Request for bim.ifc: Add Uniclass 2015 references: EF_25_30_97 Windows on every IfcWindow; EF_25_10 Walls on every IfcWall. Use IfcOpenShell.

First a look at what the model holds.

```python
import ifcopenshell

model = ifcopenshell.open("bim.ifc")
print(model.schema)
print("classifications:", [c.Name for c in model.by_type("IfcClassification")])
for ifc_class in ("IfcDoor", "IfcRoof", "IfcStair", "IfcWall", "IfcWindow"):
    print(ifc_class, len(model.by_type(ifc_class)))
```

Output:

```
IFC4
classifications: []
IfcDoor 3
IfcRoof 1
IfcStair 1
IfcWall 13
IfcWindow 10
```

```python
import ifcopenshell
import ifcopenshell.api.classification

model = ifcopenshell.open("bim.ifc")

system = ifcopenshell.api.classification.add_classification(model, classification="Uniclass 2015")

codes = {
    "IfcWindow": ("EF_25_30_97", "Windows"),
    "IfcWall": ("EF_25_10", "Walls"),
}
for ifc_class, (code, name) in codes.items():
    products = model.by_type(ifc_class)
    ifcopenshell.api.classification.add_reference(
        model, products=products, classification=system, identification=code, name=name
    )
    print(code, len(products))

model.write("bim_v2.ifc")
```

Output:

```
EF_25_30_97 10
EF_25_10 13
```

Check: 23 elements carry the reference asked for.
